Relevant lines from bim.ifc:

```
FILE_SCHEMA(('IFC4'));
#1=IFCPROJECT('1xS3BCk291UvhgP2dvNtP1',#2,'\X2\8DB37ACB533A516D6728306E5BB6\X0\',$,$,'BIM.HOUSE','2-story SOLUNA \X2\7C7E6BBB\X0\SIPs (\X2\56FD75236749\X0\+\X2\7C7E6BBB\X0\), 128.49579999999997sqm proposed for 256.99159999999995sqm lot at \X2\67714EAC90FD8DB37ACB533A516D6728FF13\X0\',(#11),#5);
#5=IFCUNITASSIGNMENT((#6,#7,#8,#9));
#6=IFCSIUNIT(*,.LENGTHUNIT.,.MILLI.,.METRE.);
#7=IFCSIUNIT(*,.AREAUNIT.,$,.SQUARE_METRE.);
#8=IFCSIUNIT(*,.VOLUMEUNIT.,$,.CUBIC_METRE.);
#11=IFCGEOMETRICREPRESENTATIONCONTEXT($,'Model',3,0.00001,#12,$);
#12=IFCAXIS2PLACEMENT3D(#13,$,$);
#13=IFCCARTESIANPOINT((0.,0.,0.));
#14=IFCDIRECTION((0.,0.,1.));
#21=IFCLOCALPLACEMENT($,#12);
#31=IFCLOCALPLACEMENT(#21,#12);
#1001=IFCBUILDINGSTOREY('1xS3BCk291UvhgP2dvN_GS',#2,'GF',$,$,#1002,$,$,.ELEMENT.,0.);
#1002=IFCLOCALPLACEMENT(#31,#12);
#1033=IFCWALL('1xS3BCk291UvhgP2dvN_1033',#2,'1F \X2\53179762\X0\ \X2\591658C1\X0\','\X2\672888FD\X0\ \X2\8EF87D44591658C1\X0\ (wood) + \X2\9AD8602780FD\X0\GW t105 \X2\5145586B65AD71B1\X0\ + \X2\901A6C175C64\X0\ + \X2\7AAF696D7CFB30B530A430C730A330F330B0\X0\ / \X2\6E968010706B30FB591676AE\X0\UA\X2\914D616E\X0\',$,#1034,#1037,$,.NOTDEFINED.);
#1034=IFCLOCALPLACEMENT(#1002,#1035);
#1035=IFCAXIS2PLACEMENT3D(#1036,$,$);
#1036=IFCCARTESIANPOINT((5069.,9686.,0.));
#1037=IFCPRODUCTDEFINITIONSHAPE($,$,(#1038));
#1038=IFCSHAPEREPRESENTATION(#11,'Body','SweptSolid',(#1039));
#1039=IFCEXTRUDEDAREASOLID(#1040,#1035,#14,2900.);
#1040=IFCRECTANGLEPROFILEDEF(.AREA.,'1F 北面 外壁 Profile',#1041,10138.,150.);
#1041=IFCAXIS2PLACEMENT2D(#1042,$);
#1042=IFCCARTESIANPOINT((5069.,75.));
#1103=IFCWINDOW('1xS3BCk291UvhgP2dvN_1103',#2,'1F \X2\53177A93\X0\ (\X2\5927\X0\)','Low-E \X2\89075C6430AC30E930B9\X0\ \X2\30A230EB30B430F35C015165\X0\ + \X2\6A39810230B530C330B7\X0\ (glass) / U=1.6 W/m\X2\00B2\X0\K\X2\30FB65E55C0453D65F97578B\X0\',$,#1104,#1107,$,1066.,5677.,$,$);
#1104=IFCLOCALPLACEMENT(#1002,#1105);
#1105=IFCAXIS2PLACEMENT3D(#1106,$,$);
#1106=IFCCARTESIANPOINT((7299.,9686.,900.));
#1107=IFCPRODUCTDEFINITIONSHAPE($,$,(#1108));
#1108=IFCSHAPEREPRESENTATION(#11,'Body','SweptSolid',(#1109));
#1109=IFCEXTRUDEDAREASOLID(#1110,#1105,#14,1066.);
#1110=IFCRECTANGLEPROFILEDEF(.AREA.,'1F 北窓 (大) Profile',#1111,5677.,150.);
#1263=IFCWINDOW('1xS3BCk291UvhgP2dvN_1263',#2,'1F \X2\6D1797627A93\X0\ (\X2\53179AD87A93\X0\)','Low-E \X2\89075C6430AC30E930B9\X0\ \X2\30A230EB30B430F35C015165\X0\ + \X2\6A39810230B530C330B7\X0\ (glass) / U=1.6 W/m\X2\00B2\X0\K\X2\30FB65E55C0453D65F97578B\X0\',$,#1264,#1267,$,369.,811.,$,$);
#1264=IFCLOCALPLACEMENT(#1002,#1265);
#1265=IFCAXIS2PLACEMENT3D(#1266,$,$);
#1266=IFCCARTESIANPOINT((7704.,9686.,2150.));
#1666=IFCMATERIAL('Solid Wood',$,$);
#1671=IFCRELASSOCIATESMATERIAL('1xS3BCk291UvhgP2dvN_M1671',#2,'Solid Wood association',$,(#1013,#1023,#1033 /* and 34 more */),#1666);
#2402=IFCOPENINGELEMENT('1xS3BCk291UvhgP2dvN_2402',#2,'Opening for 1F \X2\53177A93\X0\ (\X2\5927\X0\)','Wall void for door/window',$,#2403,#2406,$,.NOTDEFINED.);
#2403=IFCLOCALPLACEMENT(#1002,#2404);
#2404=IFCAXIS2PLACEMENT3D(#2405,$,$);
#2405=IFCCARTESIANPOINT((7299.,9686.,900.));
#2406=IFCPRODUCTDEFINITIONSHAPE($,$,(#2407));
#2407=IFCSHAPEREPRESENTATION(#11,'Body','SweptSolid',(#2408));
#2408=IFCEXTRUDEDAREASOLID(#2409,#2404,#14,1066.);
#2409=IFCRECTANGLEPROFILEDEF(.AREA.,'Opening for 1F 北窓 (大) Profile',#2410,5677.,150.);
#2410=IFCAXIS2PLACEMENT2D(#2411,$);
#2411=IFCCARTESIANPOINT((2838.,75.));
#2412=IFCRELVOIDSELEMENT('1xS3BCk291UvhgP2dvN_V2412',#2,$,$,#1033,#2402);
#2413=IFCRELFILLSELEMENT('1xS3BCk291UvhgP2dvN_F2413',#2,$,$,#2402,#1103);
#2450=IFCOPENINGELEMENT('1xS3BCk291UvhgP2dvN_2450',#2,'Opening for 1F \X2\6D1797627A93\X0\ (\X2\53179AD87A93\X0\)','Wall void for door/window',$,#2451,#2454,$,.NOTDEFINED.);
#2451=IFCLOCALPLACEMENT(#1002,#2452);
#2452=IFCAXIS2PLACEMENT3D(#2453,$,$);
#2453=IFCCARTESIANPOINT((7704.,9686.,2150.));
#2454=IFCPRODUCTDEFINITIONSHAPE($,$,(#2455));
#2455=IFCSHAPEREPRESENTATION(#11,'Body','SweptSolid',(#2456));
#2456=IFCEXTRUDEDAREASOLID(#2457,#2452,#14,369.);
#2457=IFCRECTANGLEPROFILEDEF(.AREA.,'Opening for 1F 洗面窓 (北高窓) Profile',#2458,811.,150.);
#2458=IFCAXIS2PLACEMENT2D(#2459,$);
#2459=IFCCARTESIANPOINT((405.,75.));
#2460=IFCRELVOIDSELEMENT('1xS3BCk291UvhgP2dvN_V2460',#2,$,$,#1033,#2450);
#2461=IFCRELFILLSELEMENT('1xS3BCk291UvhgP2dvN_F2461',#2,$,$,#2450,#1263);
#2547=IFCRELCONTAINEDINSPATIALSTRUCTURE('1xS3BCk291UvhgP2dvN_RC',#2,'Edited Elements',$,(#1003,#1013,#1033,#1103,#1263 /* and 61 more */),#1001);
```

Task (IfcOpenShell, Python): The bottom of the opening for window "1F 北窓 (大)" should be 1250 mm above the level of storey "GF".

```python
import numpy as np
import ifcopenshell
import ifcopenshell.api.geometry
import ifcopenshell.geom
import ifcopenshell.util.element
import ifcopenshell.util.placement
import ifcopenshell.util.shape
import ifcopenshell.util.unit

model = ifcopenshell.open("bim.ifc")
unit_scale = ifcopenshell.util.unit.calculate_unit_scale(model)

window = model.by_guid("1xS3BCk291UvhgP2dvN_1103")
opening = window.FillsVoids[0].RelatingOpeningElement
storey = ifcopenshell.util.element.get_container(window, ifc_class="IfcBuildingStorey")
level = ifcopenshell.util.placement.get_local_placement(storey.ObjectPlacement)[2, 3]

# The opening's origin need not be at the sill, so measure its lowest point.
shape = ifcopenshell.geom.create_shape(ifcopenshell.geom.settings(), opening)
bottom = ifcopenshell.util.shape.get_shape_bottom_elevation(shape, shape.geometry) / unit_scale
dz = level + 1.25 / unit_scale - bottom

shift = np.array([0.0, 0.0, dz])
# The window is not placed relative to its opening, so move both.
for product in (opening, window):
    matrix = ifcopenshell.util.placement.get_local_placement(product.ObjectPlacement)
    matrix[:3, 3] += shift
    ifcopenshell.api.geometry.edit_object_placement(model, product=product, matrix=matrix, is_si=False)

print(f"moved by {dz * unit_scale:+.3f} m")

model.write("bim_rev.ifc")
```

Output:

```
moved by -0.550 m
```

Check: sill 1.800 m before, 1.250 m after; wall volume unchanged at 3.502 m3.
